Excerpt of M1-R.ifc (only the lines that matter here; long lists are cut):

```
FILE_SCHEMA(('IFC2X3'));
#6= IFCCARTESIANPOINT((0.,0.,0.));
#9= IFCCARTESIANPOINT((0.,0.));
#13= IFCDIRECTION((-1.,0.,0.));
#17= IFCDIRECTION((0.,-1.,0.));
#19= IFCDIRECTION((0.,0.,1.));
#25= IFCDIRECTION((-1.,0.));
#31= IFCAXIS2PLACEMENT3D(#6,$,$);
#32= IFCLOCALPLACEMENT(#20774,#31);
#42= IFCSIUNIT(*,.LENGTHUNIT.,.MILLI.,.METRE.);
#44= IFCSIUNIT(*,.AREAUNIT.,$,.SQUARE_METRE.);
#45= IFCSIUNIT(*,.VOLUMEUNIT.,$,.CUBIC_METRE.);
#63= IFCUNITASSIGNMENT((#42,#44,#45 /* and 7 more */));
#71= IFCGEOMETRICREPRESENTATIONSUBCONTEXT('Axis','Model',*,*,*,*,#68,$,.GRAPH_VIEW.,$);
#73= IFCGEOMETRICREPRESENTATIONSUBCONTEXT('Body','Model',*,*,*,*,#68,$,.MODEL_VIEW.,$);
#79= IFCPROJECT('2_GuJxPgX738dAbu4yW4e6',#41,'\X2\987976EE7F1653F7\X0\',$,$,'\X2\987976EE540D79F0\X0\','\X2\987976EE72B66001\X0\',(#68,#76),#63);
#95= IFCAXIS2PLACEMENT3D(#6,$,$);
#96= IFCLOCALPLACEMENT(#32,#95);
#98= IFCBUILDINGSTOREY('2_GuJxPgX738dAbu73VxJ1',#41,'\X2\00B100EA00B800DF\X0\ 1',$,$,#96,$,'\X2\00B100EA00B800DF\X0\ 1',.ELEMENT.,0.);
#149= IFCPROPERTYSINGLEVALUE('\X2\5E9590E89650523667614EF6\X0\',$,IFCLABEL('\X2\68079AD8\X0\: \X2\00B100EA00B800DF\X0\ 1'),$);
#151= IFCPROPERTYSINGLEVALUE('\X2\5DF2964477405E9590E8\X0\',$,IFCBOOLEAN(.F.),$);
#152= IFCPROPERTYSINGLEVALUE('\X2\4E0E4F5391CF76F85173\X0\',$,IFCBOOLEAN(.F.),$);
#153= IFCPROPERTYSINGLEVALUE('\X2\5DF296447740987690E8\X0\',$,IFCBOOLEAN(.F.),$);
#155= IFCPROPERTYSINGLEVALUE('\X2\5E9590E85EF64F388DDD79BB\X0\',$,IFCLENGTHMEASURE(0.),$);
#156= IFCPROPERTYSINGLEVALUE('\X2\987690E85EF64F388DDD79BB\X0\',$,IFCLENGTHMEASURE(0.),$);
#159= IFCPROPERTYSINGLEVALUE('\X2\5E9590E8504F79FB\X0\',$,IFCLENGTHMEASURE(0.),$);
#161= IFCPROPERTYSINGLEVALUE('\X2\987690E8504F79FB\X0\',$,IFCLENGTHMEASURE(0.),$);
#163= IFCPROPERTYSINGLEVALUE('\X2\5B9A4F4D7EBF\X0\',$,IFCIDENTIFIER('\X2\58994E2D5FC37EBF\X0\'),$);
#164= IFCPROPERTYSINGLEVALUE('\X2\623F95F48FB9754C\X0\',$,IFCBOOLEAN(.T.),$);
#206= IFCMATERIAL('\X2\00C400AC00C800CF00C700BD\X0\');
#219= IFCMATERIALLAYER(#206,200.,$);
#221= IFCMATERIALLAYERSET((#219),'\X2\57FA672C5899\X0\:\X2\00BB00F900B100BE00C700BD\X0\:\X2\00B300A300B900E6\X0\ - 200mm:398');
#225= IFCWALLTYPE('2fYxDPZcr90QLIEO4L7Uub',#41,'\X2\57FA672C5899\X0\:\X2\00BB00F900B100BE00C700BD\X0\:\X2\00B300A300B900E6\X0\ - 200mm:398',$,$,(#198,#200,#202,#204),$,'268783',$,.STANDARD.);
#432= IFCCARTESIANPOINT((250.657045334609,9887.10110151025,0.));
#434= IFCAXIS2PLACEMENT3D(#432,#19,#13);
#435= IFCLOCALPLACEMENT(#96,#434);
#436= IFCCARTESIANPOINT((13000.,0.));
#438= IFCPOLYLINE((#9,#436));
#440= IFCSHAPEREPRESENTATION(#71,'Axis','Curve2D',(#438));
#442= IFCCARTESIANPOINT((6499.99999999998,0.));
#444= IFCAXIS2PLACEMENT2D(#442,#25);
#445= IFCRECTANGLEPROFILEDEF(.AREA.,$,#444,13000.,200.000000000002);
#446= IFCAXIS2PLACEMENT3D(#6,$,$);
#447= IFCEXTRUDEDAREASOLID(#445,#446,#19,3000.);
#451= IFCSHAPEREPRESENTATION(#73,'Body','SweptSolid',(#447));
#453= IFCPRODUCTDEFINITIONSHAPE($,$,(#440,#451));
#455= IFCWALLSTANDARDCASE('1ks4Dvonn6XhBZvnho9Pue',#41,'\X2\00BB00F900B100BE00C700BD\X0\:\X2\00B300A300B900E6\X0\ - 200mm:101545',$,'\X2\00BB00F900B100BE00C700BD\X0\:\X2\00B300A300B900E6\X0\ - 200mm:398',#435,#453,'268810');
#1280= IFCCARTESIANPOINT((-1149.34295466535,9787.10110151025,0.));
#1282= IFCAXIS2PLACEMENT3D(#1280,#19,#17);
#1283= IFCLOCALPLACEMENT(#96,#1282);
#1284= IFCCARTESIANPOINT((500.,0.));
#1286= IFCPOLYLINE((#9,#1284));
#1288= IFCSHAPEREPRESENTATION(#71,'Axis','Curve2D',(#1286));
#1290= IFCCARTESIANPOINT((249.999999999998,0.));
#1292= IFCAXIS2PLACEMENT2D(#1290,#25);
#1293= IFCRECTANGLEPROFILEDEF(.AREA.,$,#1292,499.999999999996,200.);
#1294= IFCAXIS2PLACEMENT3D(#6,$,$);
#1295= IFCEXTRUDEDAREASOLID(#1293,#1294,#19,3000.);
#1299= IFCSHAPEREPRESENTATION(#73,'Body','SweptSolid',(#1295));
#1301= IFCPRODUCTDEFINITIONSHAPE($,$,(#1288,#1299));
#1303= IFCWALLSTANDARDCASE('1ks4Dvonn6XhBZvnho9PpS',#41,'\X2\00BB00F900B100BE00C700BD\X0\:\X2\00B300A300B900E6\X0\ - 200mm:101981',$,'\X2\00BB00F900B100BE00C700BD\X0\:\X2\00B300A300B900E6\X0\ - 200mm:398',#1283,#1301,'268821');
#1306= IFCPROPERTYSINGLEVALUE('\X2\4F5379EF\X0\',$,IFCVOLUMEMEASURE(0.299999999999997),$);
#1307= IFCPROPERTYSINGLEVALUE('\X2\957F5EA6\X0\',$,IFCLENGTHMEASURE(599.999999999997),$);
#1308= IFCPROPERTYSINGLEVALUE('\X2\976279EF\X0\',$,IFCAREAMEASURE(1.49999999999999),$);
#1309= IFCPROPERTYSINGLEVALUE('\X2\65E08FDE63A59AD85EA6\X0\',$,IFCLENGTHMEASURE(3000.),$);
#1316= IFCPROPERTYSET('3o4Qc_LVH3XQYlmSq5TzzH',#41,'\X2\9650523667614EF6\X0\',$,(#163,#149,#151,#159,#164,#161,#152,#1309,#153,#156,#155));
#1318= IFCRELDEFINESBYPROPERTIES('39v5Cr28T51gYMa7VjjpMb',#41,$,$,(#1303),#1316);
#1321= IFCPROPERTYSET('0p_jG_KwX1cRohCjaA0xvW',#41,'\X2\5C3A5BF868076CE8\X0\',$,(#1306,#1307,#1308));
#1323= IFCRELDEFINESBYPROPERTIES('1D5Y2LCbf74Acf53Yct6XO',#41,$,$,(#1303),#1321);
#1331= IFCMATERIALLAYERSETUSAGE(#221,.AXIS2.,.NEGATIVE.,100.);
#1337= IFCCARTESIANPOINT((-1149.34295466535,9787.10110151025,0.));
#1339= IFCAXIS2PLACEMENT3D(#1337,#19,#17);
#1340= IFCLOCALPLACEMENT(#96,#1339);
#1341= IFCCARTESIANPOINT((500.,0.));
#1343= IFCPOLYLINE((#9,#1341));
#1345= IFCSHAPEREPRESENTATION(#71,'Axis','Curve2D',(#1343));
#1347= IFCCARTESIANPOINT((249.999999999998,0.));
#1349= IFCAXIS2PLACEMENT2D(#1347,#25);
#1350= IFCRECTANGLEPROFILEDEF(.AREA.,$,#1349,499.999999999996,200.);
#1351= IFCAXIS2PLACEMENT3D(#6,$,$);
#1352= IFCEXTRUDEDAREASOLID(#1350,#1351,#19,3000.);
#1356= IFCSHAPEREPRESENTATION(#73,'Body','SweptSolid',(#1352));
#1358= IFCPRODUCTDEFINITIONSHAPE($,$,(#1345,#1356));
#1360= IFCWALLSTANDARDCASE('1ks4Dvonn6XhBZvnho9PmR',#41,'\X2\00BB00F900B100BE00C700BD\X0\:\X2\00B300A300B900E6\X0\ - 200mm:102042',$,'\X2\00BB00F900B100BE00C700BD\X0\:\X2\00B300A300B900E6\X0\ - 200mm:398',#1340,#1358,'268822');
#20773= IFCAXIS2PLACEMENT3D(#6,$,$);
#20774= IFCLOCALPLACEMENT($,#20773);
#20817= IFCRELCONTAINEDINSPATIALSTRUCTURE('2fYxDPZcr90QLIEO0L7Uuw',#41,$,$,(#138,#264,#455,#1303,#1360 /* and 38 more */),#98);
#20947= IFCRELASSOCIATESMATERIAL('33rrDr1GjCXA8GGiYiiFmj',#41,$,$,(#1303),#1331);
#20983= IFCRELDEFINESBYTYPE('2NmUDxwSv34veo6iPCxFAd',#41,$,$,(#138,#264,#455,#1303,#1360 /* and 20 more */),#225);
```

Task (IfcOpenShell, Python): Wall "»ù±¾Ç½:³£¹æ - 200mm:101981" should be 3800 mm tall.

```python
import ifcopenshell
import ifcopenshell.api.pset
import ifcopenshell.geom
import ifcopenshell.util.element
import ifcopenshell.util.representation
import ifcopenshell.util.shape
import ifcopenshell.util.unit

model = ifcopenshell.open("M1-R.ifc")
unit_scale = ifcopenshell.util.unit.calculate_unit_scale(model)
area_scale = ifcopenshell.util.unit.calculate_unit_scale(model, "AREAUNIT")
volume_scale = ifcopenshell.util.unit.calculate_unit_scale(model, "VOLUMEUNIT")
settings = ifcopenshell.geom.settings()


def volume(element):
    """Net volume in cubic metres, openings subtracted."""
    shape = ifcopenshell.geom.create_shape(settings, element)
    return ifcopenshell.util.shape.get_volume(shape.geometry)


wall = model.by_guid("1ks4Dvonn6XhBZvnho9PpS")
before = volume(wall)

body = ifcopenshell.util.representation.get_representation(wall, "Model", "Body")
solid = body.Items[0]
old_height = solid.Depth
solid.Depth = 3.8 / unit_scale
after = volume(wall)
thickness = 0.2  # wall thickness in metres

# Update the stored height, areas and volumes.
pset = model.by_id(ifcopenshell.util.element.get_pset(wall, "限制条件", should_inherit=False)["id"])
ifcopenshell.api.pset.edit_pset(model, pset=pset, properties={
    "无连接高度": model.create_entity("IfcLengthMeasure", solid.Depth),
})
pset = model.by_id(ifcopenshell.util.element.get_pset(wall, "尺寸标注", should_inherit=False)["id"])
ifcopenshell.api.pset.edit_pset(model, pset=pset, properties={
    "体积": model.create_entity("IfcVolumeMeasure", after / volume_scale),
    "面积": model.create_entity("IfcAreaMeasure", after / thickness / area_scale),
})

print(f"height {old_height:g} -> {solid.Depth:g}, volume {before:.3f} -> {after:.3f} m3")

model.write("M1-R-out.ifc")
```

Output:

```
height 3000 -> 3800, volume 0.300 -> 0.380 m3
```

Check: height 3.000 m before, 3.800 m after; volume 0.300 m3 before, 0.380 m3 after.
